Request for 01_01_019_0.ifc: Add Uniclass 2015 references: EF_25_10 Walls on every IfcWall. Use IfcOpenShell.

First a look at what the model holds.

```python
import ifcopenshell

model = ifcopenshell.open("01_01_019_0.ifc")
print(model.schema)
print("classifications:", [c.Name for c in model.by_type("IfcClassification")])
for ifc_class in ("IfcDoor", "IfcRoof", "IfcStair", "IfcWall", "IfcWindow"):
    print(ifc_class, len(model.by_type(ifc_class)))
```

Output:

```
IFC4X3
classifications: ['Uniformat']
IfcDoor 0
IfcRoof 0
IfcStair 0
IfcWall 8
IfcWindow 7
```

```python
import ifcopenshell
import ifcopenshell.api.classification

model = ifcopenshell.open("01_01_019_0.ifc")

system = ifcopenshell.api.classification.add_classification(model, classification="Uniclass 2015")

codes = {
    "IfcWall": ("EF_25_10", "Walls"),
}
for ifc_class, (code, name) in codes.items():
    products = model.by_type(ifc_class)
    ifcopenshell.api.classification.add_reference(
        model, products=products, classification=system, identification=code, name=name
    )
    print(code, len(products))

model.write("01_01_019_0_edited.ifc")
```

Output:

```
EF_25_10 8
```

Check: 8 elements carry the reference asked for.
